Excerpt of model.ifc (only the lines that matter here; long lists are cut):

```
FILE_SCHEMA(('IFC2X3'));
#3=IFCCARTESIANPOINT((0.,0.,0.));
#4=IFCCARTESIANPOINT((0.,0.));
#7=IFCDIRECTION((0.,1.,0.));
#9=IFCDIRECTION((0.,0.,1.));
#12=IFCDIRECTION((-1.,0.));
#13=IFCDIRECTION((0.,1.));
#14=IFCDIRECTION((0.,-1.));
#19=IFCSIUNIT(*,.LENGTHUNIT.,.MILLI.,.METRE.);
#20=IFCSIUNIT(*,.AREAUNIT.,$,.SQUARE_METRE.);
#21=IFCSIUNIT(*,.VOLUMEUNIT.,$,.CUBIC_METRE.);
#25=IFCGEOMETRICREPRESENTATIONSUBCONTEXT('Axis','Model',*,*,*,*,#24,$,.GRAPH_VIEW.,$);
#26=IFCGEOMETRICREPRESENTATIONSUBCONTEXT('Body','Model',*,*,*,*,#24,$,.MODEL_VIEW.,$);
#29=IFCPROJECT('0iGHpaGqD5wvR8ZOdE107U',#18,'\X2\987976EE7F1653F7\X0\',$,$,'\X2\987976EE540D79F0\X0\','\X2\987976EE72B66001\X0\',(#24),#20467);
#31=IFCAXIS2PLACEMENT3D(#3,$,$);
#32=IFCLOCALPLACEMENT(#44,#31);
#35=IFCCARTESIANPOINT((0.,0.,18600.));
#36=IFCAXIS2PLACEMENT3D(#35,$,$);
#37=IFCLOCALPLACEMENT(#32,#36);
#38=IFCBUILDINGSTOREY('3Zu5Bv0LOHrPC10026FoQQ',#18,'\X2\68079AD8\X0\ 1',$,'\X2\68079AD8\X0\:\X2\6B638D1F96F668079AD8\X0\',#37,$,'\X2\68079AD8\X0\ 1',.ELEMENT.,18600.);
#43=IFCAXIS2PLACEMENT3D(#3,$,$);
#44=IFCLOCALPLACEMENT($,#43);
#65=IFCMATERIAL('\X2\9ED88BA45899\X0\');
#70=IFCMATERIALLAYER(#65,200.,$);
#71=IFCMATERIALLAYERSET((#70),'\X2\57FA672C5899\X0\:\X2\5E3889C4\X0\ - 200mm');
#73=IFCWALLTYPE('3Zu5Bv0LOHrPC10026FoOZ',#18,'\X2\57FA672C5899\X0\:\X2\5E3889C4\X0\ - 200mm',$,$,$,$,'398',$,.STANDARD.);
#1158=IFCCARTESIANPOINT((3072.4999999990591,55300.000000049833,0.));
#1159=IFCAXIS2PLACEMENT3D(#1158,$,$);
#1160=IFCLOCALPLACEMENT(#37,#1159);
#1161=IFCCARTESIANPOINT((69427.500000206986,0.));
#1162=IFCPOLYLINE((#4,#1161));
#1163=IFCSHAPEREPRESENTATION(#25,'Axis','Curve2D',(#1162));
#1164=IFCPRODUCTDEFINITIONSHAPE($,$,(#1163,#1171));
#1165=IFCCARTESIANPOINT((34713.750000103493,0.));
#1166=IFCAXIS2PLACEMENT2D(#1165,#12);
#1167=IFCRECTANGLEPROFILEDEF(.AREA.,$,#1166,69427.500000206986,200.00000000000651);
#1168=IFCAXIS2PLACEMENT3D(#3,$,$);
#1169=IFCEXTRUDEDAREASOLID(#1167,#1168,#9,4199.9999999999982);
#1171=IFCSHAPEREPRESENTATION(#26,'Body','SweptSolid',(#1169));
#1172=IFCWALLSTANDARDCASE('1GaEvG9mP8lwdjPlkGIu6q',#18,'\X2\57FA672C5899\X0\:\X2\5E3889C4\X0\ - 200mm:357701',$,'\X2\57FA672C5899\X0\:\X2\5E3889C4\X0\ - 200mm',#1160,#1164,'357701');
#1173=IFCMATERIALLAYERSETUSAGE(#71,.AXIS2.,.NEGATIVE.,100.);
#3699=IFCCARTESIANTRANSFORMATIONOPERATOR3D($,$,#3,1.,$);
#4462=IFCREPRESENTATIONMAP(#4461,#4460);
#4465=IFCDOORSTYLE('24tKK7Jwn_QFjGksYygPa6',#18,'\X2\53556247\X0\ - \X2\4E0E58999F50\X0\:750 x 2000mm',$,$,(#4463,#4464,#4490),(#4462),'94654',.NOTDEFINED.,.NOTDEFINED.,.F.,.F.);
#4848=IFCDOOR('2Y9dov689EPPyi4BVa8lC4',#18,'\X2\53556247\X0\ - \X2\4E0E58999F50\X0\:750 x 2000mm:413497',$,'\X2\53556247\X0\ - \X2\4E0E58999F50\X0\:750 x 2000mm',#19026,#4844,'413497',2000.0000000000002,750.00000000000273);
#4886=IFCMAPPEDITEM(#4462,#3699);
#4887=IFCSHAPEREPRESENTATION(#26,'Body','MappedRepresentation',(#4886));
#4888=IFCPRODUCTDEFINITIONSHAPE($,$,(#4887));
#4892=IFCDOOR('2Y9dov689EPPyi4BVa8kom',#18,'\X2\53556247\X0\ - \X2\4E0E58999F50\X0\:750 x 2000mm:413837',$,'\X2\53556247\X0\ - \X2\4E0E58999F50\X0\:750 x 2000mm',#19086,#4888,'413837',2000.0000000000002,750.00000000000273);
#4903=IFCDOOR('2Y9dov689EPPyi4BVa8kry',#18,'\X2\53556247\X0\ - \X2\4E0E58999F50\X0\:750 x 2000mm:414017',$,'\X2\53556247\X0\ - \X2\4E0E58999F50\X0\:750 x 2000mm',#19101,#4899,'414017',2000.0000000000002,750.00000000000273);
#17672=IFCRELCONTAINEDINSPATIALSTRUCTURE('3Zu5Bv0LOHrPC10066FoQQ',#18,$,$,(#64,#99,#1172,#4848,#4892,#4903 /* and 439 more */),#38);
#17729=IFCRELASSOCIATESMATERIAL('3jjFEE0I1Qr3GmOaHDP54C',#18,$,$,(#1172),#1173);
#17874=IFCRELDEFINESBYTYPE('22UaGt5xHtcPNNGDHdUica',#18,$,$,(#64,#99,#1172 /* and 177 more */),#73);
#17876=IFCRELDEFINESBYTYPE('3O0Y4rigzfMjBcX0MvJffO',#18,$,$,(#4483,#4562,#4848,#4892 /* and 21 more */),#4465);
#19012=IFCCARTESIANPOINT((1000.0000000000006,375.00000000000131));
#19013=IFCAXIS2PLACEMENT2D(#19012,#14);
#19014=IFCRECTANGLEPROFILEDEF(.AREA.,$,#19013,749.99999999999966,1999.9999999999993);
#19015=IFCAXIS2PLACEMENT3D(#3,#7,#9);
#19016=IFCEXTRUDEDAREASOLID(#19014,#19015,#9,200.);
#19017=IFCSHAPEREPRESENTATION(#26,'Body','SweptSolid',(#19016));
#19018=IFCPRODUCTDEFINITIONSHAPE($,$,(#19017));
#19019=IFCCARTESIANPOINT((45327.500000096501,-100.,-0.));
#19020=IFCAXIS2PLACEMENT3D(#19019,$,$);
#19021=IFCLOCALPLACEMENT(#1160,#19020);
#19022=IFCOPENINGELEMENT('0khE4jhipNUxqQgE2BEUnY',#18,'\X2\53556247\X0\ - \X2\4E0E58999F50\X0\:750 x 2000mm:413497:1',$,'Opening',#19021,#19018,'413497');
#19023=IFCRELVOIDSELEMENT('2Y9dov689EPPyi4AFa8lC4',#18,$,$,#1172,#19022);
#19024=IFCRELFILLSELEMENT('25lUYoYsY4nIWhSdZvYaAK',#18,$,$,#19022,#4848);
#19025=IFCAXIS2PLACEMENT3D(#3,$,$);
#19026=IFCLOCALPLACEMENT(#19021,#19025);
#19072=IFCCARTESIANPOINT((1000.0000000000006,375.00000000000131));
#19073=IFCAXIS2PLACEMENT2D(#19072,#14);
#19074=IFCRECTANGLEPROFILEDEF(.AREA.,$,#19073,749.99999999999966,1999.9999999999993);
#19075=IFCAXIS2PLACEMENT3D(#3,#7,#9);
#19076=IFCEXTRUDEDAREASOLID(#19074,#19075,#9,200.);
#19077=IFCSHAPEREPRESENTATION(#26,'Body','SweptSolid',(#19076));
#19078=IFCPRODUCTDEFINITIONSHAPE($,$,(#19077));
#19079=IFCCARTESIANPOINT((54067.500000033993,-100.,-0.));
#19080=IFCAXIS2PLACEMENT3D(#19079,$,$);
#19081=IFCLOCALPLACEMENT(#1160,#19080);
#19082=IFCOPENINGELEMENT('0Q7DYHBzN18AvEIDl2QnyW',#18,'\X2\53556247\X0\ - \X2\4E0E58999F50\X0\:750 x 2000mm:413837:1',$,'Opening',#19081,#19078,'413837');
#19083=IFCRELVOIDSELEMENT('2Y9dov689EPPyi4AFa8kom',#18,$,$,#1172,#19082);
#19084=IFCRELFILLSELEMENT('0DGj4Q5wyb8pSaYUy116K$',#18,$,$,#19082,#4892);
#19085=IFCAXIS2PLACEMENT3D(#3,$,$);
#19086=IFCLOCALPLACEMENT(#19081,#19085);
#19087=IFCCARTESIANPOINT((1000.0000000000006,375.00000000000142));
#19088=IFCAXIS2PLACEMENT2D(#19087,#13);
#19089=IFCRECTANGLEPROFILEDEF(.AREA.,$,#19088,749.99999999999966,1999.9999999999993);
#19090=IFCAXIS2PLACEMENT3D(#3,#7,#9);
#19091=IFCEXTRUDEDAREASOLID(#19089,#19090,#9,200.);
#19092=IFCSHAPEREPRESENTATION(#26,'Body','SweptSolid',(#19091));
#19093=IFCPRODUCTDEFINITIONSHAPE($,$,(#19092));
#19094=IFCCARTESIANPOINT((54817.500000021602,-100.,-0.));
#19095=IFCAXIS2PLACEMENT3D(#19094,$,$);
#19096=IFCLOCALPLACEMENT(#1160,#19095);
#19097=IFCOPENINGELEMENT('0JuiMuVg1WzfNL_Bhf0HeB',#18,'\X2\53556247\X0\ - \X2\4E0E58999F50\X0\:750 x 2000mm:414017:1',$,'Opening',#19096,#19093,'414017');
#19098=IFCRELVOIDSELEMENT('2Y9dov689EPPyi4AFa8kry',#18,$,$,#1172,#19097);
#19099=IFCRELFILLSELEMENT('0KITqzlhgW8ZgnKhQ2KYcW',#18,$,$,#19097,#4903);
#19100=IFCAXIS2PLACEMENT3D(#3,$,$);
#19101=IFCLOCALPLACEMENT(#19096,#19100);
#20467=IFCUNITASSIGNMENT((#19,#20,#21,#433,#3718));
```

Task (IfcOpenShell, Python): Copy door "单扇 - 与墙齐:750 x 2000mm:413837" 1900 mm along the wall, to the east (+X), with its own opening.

```python
import ifcopenshell
import ifcopenshell.api.feature
import ifcopenshell.api.geometry
import ifcopenshell.api.root
import ifcopenshell.geom
import ifcopenshell.util.element
import ifcopenshell.util.placement
import ifcopenshell.util.shape

model = ifcopenshell.open("model.ifc")
settings = ifcopenshell.geom.settings()


def volume(element):
    """Net volume in cubic metres, openings subtracted."""
    shape = ifcopenshell.geom.create_shape(settings, element)
    return ifcopenshell.util.shape.get_volume(shape.geometry)


def reuse_history(source, copy):
    """copy_class also copies each property set's owner history, people and application; keep the originals."""
    for rel in copy.IsDefinedBy:
        if rel.is_a("IfcRelDefinesByProperties") and (history := rel.RelatingPropertyDefinition.OwnerHistory):
            rel.RelatingPropertyDefinition.OwnerHistory = source.OwnerHistory
            ifcopenshell.util.element.remove_deep2(model, history)


door = model.by_guid("2Y9dov689EPPyi4BVa8kom")
opening = door.FillsVoids[0].RelatingOpeningElement
wall = opening.VoidsElements[0].RelatingBuildingElement
before = volume(wall)
shift = ifcopenshell.util.placement.get_local_placement(wall.ObjectPlacement)[:3, 0] * 1900.0

# copy_class copies the void relationship, type, container and properties, but no geometry.
new_opening = ifcopenshell.api.root.copy_class(model, product=opening)
new_opening.Representation = ifcopenshell.util.element.copy_deep(
    model, opening.Representation, exclude=["IfcGeometricRepresentationContext", "IfcRepresentationMap"]
)
new_opening.Name = "单扇 - 与墙齐:750 x 2000mm"
new_opening.Tag = None
new_door = ifcopenshell.api.root.copy_class(model, product=door)
new_door.Representation = ifcopenshell.util.element.copy_deep(
    model, door.Representation, exclude=["IfcGeometricRepresentationContext", "IfcRepresentationMap"]
)
new_door.Name = "单扇 - 与墙齐:750 x 2000mm"
new_door.Tag = None
reuse_history(door, new_door)
fills = ifcopenshell.api.feature.add_filling(model, opening=new_opening, element=new_door)
fills.OwnerHistory = new_door.OwnerHistory  # required in IFC2X3

for old, new in ((opening, new_opening), (door, new_door)):
    matrix = ifcopenshell.util.placement.get_local_placement(old.ObjectPlacement)
    matrix[:3, 3] += shift
    ifcopenshell.api.geometry.edit_object_placement(model, product=new, matrix=matrix, is_si=False)

after = volume(wall)

print(f"wall volume {before:.3f} -> {after:.3f} m3")

model.write("model_edited.ifc")
```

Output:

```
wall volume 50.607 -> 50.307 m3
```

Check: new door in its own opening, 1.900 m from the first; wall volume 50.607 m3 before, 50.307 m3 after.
